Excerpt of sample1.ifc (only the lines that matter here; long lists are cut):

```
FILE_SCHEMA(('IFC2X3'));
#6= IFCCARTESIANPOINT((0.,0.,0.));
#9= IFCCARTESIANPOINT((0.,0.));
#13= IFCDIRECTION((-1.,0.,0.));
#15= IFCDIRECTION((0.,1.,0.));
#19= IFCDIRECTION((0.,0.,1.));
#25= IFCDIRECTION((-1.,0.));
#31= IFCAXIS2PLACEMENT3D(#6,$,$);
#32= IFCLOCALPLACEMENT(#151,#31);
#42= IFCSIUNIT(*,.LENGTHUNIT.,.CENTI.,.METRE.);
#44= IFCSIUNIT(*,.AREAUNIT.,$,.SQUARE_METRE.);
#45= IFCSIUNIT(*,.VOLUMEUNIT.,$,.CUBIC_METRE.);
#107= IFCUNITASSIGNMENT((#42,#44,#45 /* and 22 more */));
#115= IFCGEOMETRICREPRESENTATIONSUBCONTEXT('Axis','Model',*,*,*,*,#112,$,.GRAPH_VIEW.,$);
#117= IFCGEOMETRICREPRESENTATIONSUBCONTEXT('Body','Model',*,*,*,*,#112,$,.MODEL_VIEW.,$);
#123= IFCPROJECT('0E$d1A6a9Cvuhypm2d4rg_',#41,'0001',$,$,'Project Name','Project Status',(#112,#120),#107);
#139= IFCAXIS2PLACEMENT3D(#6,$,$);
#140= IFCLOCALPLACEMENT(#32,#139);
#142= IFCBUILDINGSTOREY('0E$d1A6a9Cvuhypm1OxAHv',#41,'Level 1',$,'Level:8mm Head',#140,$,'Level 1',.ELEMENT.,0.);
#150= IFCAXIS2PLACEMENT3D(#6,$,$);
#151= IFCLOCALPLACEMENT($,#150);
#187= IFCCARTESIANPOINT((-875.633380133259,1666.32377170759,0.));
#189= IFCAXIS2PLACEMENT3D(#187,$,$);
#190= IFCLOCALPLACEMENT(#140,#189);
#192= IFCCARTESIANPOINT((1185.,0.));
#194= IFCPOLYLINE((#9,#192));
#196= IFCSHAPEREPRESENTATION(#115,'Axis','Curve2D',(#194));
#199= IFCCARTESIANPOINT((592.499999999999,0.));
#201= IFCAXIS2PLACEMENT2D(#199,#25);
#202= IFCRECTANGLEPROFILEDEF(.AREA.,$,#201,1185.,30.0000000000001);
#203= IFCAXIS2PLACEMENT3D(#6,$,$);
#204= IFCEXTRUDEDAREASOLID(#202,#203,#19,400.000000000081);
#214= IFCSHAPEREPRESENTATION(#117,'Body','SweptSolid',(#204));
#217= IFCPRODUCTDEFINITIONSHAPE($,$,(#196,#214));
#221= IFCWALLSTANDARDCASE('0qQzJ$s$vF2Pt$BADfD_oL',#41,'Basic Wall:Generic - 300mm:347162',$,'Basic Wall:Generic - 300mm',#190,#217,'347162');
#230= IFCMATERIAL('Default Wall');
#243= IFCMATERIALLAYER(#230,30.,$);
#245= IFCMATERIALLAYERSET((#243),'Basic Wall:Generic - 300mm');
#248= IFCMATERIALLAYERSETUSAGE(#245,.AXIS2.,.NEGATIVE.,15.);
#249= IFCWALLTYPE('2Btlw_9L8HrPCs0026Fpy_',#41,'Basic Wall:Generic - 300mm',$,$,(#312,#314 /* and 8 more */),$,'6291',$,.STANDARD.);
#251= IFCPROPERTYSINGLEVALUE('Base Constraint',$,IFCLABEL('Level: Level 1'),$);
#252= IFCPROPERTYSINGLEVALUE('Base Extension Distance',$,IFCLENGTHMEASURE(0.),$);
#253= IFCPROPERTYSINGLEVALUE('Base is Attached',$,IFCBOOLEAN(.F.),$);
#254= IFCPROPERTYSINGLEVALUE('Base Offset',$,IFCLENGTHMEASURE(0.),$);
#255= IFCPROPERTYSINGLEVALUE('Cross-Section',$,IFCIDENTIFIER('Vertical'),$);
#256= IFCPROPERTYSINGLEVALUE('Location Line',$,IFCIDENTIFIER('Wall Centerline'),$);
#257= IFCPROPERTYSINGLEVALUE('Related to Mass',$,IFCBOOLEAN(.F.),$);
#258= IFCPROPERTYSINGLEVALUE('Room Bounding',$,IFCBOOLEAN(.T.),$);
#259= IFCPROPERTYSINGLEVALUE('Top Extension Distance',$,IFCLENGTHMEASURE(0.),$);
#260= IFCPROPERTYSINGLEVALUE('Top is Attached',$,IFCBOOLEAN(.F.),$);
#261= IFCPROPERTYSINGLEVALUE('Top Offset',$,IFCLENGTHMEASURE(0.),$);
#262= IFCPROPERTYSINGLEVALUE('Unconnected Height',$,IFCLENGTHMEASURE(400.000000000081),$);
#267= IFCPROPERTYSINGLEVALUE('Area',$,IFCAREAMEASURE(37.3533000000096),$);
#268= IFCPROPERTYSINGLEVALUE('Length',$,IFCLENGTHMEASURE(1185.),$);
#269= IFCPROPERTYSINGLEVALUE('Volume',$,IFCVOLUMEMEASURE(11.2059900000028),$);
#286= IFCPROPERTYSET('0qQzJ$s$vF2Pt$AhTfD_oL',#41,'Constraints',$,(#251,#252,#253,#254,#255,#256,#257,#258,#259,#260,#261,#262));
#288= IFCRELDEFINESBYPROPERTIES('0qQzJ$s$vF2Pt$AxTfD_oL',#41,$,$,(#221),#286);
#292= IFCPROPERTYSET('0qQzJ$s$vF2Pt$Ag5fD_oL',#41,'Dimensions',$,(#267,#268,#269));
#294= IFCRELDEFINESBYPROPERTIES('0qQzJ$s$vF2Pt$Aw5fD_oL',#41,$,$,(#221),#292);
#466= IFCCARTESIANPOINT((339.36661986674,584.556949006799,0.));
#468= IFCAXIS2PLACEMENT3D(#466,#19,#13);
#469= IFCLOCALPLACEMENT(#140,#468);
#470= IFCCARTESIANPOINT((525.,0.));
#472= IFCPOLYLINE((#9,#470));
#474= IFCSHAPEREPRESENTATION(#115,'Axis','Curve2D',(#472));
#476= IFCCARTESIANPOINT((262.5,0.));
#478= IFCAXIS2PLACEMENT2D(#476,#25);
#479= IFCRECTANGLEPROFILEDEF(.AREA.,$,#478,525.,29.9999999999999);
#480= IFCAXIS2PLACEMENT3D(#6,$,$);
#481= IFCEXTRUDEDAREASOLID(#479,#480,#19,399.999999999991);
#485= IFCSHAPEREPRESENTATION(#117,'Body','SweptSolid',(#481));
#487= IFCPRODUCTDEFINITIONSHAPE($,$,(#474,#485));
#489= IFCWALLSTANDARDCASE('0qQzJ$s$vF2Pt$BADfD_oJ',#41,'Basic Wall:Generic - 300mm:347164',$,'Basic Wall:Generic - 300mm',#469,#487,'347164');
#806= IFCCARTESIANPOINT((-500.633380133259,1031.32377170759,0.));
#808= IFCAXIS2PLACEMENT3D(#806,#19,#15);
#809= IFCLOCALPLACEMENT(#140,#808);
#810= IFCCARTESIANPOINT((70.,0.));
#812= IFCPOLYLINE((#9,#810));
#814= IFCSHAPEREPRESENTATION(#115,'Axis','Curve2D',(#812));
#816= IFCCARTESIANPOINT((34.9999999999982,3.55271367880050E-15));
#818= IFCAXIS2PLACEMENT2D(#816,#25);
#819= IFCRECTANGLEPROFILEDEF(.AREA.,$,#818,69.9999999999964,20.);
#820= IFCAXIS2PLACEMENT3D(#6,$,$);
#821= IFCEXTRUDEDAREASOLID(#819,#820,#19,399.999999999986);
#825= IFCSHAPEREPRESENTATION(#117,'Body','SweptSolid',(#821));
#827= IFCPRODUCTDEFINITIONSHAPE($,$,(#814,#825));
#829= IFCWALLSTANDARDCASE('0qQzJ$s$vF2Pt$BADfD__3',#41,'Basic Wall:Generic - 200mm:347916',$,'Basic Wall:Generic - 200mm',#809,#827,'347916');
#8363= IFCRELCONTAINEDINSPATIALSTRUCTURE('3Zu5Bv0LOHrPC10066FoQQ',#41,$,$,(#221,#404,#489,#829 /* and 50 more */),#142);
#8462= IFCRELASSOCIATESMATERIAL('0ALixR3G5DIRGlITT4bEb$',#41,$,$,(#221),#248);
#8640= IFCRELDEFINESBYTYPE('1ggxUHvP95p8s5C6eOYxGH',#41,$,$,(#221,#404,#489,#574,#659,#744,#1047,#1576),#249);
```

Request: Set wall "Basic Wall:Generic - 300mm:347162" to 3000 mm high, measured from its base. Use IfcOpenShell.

```python
import ifcopenshell
import ifcopenshell.api.pset
import ifcopenshell.geom
import ifcopenshell.util.element
import ifcopenshell.util.representation
import ifcopenshell.util.shape
import ifcopenshell.util.unit

model = ifcopenshell.open("sample1.ifc")
unit_scale = ifcopenshell.util.unit.calculate_unit_scale(model)
area_scale = ifcopenshell.util.unit.calculate_unit_scale(model, "AREAUNIT")
volume_scale = ifcopenshell.util.unit.calculate_unit_scale(model, "VOLUMEUNIT")
settings = ifcopenshell.geom.settings()


def volume(element):
    """Net volume in cubic metres, openings subtracted."""
    shape = ifcopenshell.geom.create_shape(settings, element)
    return ifcopenshell.util.shape.get_volume(shape.geometry)


wall = model.by_guid("0qQzJ$s$vF2Pt$BADfD_oL")
before = volume(wall)

body = ifcopenshell.util.representation.get_representation(wall, "Model", "Body")
solid = body.Items[0]
old_height = solid.Depth
solid.Depth = 3 / unit_scale
after = volume(wall)
thickness = 0.3  # wall thickness in metres

# Update the stored height, areas and volumes.
pset = model.by_id(ifcopenshell.util.element.get_pset(wall, "Constraints", should_inherit=False)["id"])
ifcopenshell.api.pset.edit_pset(model, pset=pset, properties={
    "Unconnected Height": model.create_entity("IfcLengthMeasure", solid.Depth),
})
pset = model.by_id(ifcopenshell.util.element.get_pset(wall, "Dimensions", should_inherit=False)["id"])
ifcopenshell.api.pset.edit_pset(model, pset=pset, properties={
    "Area": model.create_entity("IfcAreaMeasure", after / thickness / area_scale),
    "Volume": model.create_entity("IfcVolumeMeasure", after / volume_scale),
})

print(f"height {old_height:g} -> {solid.Depth:g}, volume {before:.3f} -> {after:.3f} m3")

model.write("sample1_v2.ifc")
```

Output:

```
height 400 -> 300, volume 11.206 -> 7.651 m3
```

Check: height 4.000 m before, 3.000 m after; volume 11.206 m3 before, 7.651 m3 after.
